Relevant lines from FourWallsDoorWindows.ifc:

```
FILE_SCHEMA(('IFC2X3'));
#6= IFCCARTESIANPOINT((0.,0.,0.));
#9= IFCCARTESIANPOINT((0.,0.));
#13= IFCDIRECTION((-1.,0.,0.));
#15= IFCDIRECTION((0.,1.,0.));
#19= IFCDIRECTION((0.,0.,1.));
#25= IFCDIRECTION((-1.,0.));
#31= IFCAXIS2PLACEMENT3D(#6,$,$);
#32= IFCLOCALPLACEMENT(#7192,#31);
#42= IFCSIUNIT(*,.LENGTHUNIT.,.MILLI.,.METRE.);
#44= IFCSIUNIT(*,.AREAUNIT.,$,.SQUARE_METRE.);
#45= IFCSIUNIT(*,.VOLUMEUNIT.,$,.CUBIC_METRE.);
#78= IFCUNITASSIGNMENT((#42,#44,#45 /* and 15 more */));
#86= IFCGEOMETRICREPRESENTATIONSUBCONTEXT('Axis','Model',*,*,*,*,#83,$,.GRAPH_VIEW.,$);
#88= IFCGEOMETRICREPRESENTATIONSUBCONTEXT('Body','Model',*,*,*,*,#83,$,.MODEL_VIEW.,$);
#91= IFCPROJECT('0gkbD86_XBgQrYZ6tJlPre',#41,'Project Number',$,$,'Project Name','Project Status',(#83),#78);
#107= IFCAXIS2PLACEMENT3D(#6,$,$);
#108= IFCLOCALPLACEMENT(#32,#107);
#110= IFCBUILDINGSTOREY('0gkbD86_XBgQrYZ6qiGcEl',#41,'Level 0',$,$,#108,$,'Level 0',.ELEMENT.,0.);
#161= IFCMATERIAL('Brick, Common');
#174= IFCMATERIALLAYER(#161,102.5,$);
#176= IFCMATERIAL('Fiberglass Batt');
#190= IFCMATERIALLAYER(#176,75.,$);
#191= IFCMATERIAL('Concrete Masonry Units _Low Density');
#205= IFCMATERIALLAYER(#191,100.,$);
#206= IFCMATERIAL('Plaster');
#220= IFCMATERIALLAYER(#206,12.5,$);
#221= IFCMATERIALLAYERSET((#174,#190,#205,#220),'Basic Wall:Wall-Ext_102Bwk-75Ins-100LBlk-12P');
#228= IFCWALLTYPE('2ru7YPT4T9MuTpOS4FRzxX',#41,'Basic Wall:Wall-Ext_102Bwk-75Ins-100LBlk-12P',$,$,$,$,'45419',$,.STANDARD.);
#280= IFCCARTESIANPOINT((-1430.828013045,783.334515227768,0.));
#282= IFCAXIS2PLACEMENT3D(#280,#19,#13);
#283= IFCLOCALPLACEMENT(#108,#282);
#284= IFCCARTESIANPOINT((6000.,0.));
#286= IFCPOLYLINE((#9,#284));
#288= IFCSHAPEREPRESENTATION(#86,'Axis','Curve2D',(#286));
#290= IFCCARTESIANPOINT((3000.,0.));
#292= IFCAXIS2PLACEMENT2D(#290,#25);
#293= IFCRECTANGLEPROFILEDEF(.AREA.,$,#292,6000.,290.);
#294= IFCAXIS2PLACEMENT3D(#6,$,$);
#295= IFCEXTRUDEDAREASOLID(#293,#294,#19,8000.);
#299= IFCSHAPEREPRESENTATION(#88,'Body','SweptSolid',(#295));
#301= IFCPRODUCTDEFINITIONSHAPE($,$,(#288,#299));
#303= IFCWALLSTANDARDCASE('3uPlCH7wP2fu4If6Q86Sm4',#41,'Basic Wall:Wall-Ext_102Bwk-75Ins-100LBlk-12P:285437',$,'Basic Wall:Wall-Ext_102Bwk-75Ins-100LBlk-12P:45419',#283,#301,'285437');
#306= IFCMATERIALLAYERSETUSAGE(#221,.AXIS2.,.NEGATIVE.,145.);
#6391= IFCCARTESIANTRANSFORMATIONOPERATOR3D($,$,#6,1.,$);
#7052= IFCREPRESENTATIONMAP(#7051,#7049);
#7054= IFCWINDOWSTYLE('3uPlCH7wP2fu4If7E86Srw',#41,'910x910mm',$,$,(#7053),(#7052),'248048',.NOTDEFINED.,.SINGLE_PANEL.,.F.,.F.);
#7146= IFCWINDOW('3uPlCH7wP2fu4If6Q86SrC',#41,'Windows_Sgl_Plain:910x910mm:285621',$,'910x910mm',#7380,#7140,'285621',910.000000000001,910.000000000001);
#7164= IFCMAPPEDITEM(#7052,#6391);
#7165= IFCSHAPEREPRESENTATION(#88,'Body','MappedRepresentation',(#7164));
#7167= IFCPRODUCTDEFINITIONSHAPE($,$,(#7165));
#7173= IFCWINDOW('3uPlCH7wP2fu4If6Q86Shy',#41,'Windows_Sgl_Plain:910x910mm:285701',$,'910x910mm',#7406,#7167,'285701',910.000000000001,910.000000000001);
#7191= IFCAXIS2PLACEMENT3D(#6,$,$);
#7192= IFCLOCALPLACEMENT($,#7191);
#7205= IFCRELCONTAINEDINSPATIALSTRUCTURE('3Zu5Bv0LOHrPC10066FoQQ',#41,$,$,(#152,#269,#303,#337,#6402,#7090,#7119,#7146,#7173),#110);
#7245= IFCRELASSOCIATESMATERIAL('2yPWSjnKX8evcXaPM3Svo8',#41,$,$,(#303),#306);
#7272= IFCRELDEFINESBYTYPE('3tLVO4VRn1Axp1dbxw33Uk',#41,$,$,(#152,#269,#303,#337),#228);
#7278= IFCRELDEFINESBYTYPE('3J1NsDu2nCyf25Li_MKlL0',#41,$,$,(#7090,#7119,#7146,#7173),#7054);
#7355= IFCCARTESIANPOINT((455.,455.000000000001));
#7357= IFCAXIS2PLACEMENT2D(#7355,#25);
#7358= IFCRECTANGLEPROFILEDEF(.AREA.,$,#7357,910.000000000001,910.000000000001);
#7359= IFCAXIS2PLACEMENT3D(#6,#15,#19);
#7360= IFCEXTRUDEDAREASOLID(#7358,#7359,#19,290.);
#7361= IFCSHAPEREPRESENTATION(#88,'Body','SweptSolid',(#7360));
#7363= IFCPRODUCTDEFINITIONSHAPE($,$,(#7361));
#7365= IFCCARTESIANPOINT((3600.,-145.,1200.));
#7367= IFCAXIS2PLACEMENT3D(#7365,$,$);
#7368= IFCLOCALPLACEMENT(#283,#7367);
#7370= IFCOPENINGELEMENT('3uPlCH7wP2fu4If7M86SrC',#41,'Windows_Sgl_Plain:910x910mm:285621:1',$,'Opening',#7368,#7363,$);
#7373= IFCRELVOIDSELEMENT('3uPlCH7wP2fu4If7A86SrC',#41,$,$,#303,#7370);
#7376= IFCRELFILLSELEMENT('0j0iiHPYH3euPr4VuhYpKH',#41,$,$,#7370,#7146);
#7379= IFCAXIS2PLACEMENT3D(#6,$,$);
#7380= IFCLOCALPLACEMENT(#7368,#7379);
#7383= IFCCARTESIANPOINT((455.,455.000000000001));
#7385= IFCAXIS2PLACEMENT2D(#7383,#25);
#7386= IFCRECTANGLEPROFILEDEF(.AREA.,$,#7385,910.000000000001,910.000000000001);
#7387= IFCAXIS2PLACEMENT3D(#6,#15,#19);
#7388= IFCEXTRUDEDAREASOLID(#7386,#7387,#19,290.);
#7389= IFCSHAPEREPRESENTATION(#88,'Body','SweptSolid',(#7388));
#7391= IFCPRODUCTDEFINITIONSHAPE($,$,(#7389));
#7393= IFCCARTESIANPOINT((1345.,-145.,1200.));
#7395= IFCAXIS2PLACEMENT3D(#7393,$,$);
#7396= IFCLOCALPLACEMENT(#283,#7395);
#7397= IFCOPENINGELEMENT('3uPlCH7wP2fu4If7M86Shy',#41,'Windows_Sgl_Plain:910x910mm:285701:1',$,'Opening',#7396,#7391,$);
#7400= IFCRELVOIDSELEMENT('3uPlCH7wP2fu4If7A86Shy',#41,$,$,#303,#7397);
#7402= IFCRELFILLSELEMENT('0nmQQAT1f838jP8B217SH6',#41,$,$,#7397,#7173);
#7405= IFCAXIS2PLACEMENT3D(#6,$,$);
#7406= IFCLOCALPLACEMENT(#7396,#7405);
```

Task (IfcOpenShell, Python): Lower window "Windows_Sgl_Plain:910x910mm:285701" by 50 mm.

```python
import numpy as np
import ifcopenshell
import ifcopenshell.api.geometry
import ifcopenshell.util.placement
import ifcopenshell.util.unit

model = ifcopenshell.open("FourWallsDoorWindows.ifc")
unit_scale = ifcopenshell.util.unit.calculate_unit_scale(model)

window = model.by_guid("3uPlCH7wP2fu4If6Q86Shy")
opening = window.FillsVoids[0].RelatingOpeningElement
dz = -50.0

shift = np.array([0.0, 0.0, dz])
# The window is placed relative to its opening, so it follows when the opening moves.
matrix = ifcopenshell.util.placement.get_local_placement(opening.ObjectPlacement)
matrix[:3, 3] += shift
ifcopenshell.api.geometry.edit_object_placement(
    model, product=opening, matrix=matrix, is_si=False, should_transform_children=True
)

print(f"moved by {dz * unit_scale:+.3f} m")

model.write("FourWallsDoorWindows_edited.ifc")
```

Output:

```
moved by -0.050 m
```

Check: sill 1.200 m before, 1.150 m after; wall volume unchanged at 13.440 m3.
